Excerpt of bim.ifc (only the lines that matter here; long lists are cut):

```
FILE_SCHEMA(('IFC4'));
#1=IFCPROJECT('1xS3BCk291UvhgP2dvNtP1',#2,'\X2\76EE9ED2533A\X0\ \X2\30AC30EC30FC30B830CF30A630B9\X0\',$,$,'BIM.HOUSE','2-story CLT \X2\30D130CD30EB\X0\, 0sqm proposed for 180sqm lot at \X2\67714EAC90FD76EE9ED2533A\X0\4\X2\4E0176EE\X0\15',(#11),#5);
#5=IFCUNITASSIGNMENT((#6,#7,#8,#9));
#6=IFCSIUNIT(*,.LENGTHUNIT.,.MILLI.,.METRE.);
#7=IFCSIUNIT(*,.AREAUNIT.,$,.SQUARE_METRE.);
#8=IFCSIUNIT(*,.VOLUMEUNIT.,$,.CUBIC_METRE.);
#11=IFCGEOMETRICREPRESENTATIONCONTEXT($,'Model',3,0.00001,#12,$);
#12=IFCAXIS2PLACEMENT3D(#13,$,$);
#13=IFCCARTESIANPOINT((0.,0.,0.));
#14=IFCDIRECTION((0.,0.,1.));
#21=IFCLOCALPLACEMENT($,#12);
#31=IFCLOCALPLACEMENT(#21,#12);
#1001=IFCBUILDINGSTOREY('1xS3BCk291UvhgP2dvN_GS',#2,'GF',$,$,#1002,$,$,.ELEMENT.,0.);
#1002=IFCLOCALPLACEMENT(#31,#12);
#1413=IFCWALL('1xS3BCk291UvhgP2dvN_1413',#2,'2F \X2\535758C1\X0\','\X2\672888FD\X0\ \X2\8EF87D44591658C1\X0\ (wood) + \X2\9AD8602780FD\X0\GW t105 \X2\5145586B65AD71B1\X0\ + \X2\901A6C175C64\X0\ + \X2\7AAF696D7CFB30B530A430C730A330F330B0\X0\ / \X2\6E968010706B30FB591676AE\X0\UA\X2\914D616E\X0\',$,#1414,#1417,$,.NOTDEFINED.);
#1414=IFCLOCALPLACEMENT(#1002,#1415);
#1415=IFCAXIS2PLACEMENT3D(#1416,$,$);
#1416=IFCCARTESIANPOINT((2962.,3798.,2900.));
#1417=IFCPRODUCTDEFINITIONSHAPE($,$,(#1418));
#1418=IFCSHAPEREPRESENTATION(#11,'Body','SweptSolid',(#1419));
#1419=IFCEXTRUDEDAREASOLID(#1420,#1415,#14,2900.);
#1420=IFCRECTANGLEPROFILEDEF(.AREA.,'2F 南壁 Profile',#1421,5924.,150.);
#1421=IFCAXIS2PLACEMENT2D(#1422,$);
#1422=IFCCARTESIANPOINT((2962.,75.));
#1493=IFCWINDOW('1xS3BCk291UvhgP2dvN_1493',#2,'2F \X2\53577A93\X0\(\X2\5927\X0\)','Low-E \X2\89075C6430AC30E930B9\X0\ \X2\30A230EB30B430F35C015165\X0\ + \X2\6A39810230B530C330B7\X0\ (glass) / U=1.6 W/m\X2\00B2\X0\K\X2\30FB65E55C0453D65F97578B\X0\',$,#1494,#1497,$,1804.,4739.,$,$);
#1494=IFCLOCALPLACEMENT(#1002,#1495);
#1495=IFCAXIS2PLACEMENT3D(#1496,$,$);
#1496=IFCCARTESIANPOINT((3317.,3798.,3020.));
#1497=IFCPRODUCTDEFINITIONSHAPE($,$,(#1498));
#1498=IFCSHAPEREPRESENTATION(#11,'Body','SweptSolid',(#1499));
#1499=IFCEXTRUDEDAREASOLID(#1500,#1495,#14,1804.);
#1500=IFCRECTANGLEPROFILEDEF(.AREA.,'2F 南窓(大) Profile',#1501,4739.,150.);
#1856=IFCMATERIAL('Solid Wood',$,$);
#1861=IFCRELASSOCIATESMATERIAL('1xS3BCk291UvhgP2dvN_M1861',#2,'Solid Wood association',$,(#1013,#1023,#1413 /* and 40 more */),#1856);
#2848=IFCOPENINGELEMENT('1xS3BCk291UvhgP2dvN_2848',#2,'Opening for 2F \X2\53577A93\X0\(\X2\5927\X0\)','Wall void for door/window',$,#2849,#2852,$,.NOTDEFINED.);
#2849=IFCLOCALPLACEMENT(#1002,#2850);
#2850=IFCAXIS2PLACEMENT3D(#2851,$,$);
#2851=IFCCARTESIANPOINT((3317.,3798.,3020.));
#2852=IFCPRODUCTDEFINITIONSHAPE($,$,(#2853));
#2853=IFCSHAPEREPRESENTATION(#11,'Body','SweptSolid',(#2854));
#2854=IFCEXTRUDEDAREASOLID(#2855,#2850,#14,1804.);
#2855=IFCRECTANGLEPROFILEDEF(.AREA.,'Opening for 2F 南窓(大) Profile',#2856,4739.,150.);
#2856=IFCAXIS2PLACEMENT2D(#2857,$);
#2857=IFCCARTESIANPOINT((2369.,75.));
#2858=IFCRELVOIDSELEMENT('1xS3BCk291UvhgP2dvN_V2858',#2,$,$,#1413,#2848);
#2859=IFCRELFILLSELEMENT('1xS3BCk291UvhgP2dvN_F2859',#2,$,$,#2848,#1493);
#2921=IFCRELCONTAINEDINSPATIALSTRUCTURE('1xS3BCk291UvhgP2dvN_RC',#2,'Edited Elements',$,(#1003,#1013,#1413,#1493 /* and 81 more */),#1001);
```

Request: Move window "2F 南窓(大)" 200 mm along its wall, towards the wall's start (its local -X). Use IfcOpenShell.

```python
import ifcopenshell
import ifcopenshell.api.geometry
import ifcopenshell.util.placement
import ifcopenshell.util.unit

model = ifcopenshell.open("bim.ifc")
unit_scale = ifcopenshell.util.unit.calculate_unit_scale(model)

window = model.by_id(1493)
opening = window.FillsVoids[0].RelatingOpeningElement
wall = opening.VoidsElements[0].RelatingBuildingElement

wall_matrix = ifcopenshell.util.placement.get_local_placement(wall.ObjectPlacement)
shift = wall_matrix[:3, 0] * -0.2 / unit_scale
before = ifcopenshell.util.placement.get_local_placement(window.ObjectPlacement)[:3, 3].copy()

# The window is not placed relative to its opening, so move both.
for product in (opening, window):
    matrix = ifcopenshell.util.placement.get_local_placement(product.ObjectPlacement)
    matrix[:3, 3] += shift
    ifcopenshell.api.geometry.edit_object_placement(model, product=product, matrix=matrix, is_si=False)

after = ifcopenshell.util.placement.get_local_placement(window.ObjectPlacement)[:3, 3]
print("window moved by", (after - before).round(3) + 0.0)

model.write("bim_edited.ifc")
```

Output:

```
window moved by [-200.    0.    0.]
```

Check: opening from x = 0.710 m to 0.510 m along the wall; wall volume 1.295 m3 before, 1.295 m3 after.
